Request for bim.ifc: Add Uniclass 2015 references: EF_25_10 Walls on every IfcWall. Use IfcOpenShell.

First a look at what the model holds.

```python
import ifcopenshell

model = ifcopenshell.open("bim.ifc")
print(model.schema)
print("classifications:", [c.Name for c in model.by_type("IfcClassification")])
for ifc_class in ("IfcDoor", "IfcRoof", "IfcStair", "IfcWall", "IfcWindow"):
    print(ifc_class, len(model.by_type(ifc_class)))
```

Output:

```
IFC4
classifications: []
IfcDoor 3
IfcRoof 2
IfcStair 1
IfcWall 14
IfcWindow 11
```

```python
import ifcopenshell
import ifcopenshell.api.classification

model = ifcopenshell.open("bim.ifc")

system = ifcopenshell.api.classification.add_classification(model, classification="Uniclass 2015")

codes = {
    "IfcWall": ("EF_25_10", "Walls"),
}
for ifc_class, (code, name) in codes.items():
    products = model.by_type(ifc_class)
    ifcopenshell.api.classification.add_reference(
        model, products=products, classification=system, identification=code, name=name
    )
    print(code, len(products))

model.write("bim_rev.ifc")
```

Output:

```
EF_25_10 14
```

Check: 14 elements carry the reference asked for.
